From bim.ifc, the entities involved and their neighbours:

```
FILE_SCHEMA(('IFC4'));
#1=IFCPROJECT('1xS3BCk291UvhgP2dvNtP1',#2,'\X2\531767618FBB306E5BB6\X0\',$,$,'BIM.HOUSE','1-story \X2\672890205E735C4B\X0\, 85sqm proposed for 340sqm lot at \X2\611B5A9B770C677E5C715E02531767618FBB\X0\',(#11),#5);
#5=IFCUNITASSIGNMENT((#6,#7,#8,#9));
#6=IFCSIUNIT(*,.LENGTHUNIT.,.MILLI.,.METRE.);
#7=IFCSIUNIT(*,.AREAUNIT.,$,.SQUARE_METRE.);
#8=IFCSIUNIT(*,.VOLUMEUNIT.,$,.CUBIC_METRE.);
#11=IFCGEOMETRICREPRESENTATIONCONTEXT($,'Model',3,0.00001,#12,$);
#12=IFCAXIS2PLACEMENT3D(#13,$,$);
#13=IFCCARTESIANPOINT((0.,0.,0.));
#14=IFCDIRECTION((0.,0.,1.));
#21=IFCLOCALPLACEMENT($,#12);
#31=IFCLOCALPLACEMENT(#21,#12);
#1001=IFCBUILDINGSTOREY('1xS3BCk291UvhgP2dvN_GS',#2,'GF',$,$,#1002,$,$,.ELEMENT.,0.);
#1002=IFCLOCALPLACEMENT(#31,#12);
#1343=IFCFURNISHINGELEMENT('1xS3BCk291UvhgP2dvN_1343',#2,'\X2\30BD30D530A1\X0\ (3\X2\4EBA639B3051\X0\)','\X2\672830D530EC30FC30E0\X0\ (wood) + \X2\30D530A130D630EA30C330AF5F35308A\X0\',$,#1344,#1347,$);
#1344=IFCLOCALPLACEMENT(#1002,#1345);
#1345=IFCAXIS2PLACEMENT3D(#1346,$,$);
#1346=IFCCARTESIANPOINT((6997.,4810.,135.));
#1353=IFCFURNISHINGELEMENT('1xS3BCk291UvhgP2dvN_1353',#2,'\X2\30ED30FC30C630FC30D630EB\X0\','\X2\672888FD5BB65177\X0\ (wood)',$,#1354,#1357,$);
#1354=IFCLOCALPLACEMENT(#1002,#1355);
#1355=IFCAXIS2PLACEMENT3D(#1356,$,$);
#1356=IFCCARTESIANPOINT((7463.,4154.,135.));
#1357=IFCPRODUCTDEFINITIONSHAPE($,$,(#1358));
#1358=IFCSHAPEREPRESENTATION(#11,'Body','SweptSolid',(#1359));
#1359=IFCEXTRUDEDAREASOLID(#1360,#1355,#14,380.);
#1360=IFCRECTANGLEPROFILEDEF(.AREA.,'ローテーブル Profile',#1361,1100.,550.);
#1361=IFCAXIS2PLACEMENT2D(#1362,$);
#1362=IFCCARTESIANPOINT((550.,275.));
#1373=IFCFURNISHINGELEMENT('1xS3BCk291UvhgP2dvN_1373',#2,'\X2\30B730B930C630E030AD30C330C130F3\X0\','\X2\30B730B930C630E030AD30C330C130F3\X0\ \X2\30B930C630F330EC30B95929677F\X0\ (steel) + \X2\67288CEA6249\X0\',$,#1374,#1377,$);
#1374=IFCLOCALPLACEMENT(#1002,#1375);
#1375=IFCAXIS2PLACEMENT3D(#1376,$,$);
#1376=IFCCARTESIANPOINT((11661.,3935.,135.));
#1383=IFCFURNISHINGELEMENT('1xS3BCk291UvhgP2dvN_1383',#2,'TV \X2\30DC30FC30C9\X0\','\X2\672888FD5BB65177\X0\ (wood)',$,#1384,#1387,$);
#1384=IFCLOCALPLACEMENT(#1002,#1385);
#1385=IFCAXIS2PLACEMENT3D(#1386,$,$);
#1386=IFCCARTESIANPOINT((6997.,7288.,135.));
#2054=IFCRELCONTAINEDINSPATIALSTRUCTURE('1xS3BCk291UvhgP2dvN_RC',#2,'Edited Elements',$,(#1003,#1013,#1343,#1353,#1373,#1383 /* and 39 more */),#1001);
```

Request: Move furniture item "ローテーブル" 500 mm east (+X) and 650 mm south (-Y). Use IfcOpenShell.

```python
import ifcopenshell
import ifcopenshell.api.geometry
import ifcopenshell.util.placement

model = ifcopenshell.open("bim.ifc")

item = model.by_guid("1xS3BCk291UvhgP2dvN_1353")
matrix = ifcopenshell.util.placement.get_local_placement(item.ObjectPlacement)
matrix[0, 3] += 500.0
matrix[1, 3] -= 650.0
ifcopenshell.api.geometry.edit_object_placement(model, product=item, matrix=matrix, is_si=False)

print(ifcopenshell.util.placement.get_local_placement(item.ObjectPlacement).round(3) + 0.0)

model.write("bim_edited.ifc")
```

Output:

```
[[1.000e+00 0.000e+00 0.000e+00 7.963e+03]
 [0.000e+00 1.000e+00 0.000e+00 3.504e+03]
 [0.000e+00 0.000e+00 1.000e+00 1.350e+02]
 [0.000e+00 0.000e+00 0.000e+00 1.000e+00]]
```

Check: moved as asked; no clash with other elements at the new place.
